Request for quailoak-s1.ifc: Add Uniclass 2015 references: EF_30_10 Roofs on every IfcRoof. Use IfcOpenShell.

First a look at what the model holds.

```python
import ifcopenshell

model = ifcopenshell.open("quailoak-s1.ifc")
print(model.schema)
print("classifications:", [c.Name for c in model.by_type("IfcClassification")])
for ifc_class in ("IfcDoor", "IfcRoof", "IfcStair", "IfcWall", "IfcWindow"):
    print(ifc_class, len(model.by_type(ifc_class)))
```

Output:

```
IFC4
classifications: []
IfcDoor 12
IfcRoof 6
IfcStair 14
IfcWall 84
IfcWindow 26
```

```python
import ifcopenshell
import ifcopenshell.api.classification

model = ifcopenshell.open("quailoak-s1.ifc")

system = ifcopenshell.api.classification.add_classification(model, classification="Uniclass 2015")

codes = {
    "IfcRoof": ("EF_30_10", "Roofs"),
}
for ifc_class, (code, name) in codes.items():
    products = model.by_type(ifc_class)
    ifcopenshell.api.classification.add_reference(
        model, products=products, classification=system, identification=code, name=name
    )
    print(code, len(products))

model.write("quailoak-s1_edited.ifc")
```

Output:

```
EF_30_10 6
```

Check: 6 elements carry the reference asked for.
